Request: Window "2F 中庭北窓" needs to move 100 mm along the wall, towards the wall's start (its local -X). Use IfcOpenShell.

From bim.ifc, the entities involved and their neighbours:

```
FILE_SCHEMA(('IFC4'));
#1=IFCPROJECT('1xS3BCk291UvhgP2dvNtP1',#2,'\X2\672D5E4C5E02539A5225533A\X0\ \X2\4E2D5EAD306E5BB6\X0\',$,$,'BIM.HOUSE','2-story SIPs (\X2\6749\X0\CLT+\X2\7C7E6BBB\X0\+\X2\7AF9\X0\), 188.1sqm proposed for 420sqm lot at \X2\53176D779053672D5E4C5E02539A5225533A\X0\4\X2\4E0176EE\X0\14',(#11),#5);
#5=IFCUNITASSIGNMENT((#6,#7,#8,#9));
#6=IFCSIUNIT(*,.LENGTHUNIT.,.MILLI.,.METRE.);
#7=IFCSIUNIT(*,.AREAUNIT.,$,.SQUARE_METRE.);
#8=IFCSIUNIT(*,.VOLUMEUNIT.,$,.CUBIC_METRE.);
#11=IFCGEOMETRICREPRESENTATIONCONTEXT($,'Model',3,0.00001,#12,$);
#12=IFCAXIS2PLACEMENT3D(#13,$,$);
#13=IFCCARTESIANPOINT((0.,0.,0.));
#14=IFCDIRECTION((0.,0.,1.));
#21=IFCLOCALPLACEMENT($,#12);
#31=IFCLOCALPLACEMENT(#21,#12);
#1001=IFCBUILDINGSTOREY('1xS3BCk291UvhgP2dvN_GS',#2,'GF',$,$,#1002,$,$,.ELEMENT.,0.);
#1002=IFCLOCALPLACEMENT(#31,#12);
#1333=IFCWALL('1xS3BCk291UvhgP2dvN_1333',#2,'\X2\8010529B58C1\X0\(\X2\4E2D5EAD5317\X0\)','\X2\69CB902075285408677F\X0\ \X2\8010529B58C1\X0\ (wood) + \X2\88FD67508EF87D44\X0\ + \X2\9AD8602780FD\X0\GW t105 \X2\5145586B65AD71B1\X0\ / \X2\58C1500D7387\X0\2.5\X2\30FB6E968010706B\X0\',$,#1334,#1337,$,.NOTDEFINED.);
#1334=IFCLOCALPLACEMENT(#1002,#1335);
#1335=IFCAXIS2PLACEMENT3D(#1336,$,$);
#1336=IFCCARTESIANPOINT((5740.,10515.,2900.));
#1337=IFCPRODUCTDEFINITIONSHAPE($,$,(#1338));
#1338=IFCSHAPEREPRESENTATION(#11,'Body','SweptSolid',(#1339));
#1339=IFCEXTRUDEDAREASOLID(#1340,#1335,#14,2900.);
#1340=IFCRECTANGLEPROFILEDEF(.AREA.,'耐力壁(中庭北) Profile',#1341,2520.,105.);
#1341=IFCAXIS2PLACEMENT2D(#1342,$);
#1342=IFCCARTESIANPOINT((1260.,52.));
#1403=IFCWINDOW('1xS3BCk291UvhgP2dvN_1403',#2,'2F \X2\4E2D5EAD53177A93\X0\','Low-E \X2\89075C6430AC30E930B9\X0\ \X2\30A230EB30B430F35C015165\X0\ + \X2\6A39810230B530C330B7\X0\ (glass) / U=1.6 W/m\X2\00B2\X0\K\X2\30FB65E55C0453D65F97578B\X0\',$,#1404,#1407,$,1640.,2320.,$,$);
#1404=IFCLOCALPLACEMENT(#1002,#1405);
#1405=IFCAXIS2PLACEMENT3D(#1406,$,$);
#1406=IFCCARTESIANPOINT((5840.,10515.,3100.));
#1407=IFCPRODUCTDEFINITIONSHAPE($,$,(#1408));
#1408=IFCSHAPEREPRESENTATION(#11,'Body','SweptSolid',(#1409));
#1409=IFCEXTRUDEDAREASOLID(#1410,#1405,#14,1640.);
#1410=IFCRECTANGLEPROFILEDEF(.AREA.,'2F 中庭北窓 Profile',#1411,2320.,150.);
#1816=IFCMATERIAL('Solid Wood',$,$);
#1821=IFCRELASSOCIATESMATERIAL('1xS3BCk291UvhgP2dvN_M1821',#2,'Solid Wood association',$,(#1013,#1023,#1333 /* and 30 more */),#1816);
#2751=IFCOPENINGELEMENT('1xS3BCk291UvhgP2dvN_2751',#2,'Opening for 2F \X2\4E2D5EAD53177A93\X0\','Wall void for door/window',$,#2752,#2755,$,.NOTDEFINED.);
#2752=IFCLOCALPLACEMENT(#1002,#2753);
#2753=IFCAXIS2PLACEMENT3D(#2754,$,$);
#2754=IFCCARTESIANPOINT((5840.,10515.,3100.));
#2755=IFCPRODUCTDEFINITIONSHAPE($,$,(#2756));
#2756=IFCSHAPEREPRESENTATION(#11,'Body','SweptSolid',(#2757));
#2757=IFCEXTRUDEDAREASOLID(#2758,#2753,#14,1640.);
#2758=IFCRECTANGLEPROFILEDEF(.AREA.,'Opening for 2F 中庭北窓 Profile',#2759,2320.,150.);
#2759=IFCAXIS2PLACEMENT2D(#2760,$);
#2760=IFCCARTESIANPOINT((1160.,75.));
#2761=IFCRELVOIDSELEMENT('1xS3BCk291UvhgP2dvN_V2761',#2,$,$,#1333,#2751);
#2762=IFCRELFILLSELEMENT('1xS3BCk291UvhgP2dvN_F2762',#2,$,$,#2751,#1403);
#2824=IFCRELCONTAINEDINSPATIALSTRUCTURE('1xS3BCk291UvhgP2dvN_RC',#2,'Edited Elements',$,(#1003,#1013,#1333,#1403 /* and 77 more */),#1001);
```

```python
import ifcopenshell
import ifcopenshell.api.geometry
import ifcopenshell.util.placement
import ifcopenshell.util.unit

model = ifcopenshell.open("bim.ifc")
unit_scale = ifcopenshell.util.unit.calculate_unit_scale(model)

window = model.by_id(1403)
opening = window.FillsVoids[0].RelatingOpeningElement
wall = opening.VoidsElements[0].RelatingBuildingElement

wall_matrix = ifcopenshell.util.placement.get_local_placement(wall.ObjectPlacement)
shift = wall_matrix[:3, 0] * -0.1 / unit_scale
before = ifcopenshell.util.placement.get_local_placement(window.ObjectPlacement)[:3, 3].copy()

# The window is not placed relative to its opening, so move both.
for product in (opening, window):
    matrix = ifcopenshell.util.placement.get_local_placement(product.ObjectPlacement)
    matrix[:3, 3] += shift
    ifcopenshell.api.geometry.edit_object_placement(model, product=product, matrix=matrix, is_si=False)

after = ifcopenshell.util.placement.get_local_placement(window.ObjectPlacement)[:3, 3]
print("window moved by", (after - before).round(3) + 0.0)

model.write("bim-out.ifc")
```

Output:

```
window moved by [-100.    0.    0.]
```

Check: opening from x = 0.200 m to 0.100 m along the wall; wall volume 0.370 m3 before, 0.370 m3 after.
